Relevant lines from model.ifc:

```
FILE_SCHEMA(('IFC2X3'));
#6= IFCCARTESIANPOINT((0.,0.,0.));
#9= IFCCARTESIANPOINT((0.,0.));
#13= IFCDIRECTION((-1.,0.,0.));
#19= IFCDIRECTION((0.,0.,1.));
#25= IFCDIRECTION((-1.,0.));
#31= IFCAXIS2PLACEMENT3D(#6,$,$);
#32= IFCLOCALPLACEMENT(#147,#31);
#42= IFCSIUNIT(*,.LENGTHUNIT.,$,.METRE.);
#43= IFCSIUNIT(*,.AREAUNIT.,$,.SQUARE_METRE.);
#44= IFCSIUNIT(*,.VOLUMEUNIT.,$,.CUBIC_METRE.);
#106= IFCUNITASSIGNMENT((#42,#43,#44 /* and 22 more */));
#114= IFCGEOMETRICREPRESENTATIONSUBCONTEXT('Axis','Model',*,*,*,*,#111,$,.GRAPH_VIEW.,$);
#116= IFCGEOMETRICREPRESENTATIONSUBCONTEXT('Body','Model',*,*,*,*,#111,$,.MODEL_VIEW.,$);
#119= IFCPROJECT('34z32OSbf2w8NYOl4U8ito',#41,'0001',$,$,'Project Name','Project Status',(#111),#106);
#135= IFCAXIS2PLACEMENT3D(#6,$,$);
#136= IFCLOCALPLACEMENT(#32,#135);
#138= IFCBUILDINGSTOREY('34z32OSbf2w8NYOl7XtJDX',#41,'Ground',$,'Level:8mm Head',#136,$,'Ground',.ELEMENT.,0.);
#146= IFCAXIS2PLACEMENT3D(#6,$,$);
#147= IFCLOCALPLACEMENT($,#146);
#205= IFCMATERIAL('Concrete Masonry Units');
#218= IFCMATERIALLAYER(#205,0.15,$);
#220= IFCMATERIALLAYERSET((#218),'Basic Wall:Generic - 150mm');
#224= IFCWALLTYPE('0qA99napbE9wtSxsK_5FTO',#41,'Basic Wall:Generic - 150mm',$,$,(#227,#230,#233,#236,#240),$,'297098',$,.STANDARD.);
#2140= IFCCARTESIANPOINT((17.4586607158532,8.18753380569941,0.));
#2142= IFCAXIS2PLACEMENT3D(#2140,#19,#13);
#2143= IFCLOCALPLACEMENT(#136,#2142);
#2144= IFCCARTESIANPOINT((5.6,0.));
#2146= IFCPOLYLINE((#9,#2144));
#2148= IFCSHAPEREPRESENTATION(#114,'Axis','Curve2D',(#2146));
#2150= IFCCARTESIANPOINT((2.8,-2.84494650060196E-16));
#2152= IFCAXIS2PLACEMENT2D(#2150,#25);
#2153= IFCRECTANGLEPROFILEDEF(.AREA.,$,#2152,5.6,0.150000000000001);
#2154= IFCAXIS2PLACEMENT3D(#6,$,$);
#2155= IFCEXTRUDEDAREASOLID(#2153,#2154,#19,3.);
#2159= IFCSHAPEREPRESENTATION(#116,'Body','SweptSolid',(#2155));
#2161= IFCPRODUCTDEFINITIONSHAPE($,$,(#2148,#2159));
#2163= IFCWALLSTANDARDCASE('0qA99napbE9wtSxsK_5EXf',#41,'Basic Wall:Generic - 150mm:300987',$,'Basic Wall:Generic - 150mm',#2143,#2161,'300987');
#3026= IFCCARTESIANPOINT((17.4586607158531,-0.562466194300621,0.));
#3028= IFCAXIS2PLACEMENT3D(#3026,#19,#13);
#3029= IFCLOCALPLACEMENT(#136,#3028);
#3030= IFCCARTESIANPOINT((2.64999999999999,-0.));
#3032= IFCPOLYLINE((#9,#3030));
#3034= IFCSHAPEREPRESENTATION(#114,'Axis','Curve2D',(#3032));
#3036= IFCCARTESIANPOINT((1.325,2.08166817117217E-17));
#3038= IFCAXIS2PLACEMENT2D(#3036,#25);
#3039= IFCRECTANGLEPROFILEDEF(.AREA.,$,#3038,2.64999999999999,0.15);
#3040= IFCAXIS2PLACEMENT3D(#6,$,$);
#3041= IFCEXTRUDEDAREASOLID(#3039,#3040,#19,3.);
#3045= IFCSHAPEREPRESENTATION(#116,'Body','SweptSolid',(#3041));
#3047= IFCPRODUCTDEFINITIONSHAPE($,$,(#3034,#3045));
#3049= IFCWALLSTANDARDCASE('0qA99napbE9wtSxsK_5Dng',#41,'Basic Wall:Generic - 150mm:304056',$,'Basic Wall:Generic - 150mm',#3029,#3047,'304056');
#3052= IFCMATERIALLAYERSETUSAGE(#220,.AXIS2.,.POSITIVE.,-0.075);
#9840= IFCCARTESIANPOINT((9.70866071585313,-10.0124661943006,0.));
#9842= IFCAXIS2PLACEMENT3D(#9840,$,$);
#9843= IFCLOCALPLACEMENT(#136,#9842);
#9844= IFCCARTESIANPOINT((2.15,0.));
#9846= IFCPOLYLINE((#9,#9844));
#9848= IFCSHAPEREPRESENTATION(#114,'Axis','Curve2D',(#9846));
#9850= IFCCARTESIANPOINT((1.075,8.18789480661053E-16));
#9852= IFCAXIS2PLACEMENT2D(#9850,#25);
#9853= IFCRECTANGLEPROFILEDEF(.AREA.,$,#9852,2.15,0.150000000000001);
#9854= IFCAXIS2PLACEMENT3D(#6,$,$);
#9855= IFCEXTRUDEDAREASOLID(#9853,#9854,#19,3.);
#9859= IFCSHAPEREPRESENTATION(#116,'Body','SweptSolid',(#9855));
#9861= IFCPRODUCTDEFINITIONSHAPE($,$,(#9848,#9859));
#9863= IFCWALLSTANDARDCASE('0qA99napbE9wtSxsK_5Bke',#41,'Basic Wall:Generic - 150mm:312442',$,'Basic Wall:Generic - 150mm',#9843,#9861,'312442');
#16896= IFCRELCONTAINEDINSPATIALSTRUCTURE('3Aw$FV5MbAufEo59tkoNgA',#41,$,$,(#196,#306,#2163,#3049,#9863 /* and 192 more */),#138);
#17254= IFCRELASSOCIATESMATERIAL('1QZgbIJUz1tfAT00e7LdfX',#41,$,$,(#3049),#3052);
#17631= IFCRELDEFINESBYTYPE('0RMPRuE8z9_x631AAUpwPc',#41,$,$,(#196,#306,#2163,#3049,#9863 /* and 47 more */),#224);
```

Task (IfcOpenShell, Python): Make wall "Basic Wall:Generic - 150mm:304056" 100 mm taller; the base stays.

```python
import ifcopenshell
import ifcopenshell.geom
import ifcopenshell.util.representation
import ifcopenshell.util.shape

model = ifcopenshell.open("model.ifc")
settings = ifcopenshell.geom.settings()


def volume(element):
    """Net volume in cubic metres, openings subtracted."""
    shape = ifcopenshell.geom.create_shape(settings, element)
    return ifcopenshell.util.shape.get_volume(shape.geometry)


wall = model.by_guid("0qA99napbE9wtSxsK_5Dng")
before = volume(wall)

body = ifcopenshell.util.representation.get_representation(wall, "Model", "Body")
solid = body.Items[0]
old_height = solid.Depth
solid.Depth += 0.1
after = volume(wall)

print(f"height {old_height:g} -> {solid.Depth:g}, volume {before:.3f} -> {after:.3f} m3")

model.write("model_rev.ifc")
```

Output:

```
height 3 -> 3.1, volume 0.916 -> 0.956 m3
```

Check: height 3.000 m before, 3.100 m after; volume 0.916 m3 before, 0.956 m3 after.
